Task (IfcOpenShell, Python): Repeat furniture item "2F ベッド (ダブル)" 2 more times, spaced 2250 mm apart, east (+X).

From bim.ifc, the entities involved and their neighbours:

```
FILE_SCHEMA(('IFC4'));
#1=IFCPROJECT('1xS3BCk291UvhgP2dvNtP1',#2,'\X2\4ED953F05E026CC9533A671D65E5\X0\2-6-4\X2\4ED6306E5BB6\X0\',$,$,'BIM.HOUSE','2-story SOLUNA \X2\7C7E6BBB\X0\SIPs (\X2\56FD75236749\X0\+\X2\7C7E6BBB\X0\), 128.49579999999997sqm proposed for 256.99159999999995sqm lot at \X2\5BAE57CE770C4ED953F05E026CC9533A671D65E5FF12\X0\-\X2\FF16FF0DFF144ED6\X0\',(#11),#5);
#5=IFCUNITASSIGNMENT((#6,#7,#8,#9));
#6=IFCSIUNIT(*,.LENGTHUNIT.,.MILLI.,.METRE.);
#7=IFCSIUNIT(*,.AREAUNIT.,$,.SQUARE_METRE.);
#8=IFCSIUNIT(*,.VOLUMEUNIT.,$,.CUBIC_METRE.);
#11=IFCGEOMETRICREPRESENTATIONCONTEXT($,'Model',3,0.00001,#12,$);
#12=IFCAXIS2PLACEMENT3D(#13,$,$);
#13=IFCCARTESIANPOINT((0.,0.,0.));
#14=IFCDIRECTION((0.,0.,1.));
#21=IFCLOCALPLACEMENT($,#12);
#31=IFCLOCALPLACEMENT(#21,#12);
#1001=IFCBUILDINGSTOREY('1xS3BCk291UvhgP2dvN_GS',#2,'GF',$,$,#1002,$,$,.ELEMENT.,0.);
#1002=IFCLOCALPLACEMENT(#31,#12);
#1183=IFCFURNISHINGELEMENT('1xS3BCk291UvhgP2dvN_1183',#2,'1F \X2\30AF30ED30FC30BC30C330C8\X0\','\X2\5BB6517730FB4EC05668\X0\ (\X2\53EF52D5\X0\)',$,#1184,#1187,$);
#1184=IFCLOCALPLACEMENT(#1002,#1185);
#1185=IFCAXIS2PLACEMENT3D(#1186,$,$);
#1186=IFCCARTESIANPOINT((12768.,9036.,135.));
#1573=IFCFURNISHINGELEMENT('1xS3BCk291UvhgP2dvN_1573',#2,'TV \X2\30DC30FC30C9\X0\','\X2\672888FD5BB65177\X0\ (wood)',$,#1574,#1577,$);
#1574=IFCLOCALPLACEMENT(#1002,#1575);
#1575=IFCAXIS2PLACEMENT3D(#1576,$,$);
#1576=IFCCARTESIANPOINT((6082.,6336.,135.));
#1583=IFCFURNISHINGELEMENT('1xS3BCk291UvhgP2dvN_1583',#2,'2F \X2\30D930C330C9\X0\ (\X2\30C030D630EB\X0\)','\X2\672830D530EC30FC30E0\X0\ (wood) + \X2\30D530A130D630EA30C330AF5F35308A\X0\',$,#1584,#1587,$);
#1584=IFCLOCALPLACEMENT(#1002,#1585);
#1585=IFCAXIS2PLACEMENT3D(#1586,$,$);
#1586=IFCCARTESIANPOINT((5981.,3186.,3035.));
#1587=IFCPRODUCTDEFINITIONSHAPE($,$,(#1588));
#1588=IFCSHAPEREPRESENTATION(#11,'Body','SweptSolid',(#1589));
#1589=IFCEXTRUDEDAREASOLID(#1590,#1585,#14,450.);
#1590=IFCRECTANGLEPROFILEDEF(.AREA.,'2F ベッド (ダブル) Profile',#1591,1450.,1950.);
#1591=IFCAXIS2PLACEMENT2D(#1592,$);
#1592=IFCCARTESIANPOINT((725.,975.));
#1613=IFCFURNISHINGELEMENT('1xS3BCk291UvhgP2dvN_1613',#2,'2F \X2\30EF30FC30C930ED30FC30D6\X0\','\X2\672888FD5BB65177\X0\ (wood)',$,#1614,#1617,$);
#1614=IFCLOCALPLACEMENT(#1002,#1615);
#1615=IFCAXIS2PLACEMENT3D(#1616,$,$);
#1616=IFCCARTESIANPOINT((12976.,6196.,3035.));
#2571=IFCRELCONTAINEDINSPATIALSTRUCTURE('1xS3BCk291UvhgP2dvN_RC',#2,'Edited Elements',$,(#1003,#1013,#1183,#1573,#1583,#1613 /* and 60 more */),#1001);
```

```python
import numpy as np
import ifcopenshell
import ifcopenshell.api.geometry
import ifcopenshell.api.root
import ifcopenshell.util.element
import ifcopenshell.util.placement
import ifcopenshell.util.unit

model = ifcopenshell.open("bim.ifc")
unit_scale = ifcopenshell.util.unit.calculate_unit_scale(model)


def reuse_history(source, copy):
    """copy_class also copies each property set's owner history, people and application; keep the originals."""
    for rel in copy.IsDefinedBy:
        if rel.is_a("IfcRelDefinesByProperties") and (history := rel.RelatingPropertyDefinition.OwnerHistory):
            rel.RelatingPropertyDefinition.OwnerHistory = source.OwnerHistory
            ifcopenshell.util.element.remove_deep2(model, history)


source = model.by_id(1583)
base = ifcopenshell.util.placement.get_local_placement(source.ObjectPlacement)
step = np.array([1.0, 0.0, 0.0]) * 2.25 / unit_scale

for i in range(1, 3):
    copy = ifcopenshell.api.root.copy_class(model, product=source)
    copy.Representation = ifcopenshell.util.element.copy_deep(
        model, source.Representation, exclude=["IfcGeometricRepresentationContext", "IfcRepresentationMap"]
    )
    reuse_history(source, copy)
    matrix = base.copy()
    matrix[:3, 3] += i * step
    print("added at", matrix[:3, 3].round(3) + 0.0)
    ifcopenshell.api.geometry.edit_object_placement(model, product=copy, matrix=matrix, is_si=False)

model.write("bim_v2.ifc")
```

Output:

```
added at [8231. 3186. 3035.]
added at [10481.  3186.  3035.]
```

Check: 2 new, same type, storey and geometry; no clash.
